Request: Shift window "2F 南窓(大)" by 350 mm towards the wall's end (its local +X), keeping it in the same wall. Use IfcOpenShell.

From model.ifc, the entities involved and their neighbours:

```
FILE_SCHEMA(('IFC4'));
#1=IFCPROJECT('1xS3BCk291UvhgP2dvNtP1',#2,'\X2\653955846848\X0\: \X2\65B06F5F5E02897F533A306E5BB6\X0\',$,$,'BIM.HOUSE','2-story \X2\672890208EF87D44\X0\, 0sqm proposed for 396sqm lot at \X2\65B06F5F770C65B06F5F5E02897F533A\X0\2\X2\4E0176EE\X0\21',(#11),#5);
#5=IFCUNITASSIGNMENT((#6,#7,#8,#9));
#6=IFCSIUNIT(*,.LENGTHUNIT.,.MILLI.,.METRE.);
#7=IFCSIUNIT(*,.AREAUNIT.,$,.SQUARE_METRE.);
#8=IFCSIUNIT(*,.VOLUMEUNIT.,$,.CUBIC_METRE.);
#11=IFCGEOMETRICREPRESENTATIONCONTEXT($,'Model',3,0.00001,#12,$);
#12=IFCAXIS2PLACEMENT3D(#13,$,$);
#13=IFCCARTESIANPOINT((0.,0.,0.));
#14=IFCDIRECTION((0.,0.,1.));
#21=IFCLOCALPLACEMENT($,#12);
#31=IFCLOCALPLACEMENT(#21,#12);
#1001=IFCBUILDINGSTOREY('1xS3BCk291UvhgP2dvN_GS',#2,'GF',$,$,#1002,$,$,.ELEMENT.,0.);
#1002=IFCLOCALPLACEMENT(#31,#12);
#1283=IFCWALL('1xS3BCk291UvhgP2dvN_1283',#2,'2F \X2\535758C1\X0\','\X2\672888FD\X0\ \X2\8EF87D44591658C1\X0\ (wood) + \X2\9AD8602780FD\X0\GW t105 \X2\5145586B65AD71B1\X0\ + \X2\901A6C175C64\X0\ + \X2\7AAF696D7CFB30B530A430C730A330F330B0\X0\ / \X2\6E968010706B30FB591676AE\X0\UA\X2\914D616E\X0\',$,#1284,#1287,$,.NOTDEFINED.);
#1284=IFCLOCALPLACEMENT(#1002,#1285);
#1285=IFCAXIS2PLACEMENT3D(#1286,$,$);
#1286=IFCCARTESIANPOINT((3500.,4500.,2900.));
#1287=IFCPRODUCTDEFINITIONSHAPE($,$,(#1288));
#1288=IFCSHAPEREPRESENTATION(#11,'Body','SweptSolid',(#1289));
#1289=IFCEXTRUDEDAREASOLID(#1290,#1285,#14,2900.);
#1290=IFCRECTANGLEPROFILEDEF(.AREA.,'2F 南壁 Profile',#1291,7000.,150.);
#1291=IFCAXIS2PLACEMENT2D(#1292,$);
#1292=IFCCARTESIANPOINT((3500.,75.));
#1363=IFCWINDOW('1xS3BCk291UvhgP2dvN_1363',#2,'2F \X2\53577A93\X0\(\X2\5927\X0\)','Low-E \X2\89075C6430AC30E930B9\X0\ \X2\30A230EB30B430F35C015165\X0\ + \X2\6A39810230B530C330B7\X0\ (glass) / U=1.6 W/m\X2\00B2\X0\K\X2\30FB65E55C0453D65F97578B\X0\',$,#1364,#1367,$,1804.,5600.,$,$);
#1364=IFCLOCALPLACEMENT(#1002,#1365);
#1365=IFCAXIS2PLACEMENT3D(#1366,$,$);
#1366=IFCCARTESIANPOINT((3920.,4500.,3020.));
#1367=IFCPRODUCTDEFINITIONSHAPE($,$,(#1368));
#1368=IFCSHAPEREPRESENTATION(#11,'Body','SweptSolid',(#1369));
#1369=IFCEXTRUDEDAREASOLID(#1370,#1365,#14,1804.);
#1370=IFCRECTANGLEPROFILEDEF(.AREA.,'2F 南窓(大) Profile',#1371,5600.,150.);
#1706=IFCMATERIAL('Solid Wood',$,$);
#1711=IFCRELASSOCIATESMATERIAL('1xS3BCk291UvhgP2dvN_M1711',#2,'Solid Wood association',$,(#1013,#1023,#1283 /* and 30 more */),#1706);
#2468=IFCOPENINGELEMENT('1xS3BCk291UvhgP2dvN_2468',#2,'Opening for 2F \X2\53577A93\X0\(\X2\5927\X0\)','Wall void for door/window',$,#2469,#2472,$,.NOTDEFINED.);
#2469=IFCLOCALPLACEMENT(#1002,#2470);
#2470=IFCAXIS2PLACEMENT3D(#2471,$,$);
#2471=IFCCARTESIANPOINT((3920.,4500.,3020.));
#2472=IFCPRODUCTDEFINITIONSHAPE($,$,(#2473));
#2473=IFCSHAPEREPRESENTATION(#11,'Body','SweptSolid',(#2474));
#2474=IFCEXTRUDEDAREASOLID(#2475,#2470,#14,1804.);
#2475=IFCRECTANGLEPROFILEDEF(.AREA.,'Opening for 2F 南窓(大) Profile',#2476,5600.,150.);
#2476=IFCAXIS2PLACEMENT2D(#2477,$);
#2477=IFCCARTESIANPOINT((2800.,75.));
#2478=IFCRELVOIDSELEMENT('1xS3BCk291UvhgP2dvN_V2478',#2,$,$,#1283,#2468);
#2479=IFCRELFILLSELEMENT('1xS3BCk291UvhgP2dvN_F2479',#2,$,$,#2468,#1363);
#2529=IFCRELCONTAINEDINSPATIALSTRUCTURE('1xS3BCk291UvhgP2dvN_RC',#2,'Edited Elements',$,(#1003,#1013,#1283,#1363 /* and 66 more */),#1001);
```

```python
import ifcopenshell
import ifcopenshell.api.geometry
import ifcopenshell.util.placement

model = ifcopenshell.open("model.ifc")

window = model.by_guid("1xS3BCk291UvhgP2dvN_1363")
opening = window.FillsVoids[0].RelatingOpeningElement
wall = opening.VoidsElements[0].RelatingBuildingElement

wall_matrix = ifcopenshell.util.placement.get_local_placement(wall.ObjectPlacement)
shift = wall_matrix[:3, 0] * 350.0
before = ifcopenshell.util.placement.get_local_placement(window.ObjectPlacement)[:3, 3].copy()

# The window is not placed relative to its opening, so move both.
for product in (opening, window):
    matrix = ifcopenshell.util.placement.get_local_placement(product.ObjectPlacement)
    matrix[:3, 3] += shift
    ifcopenshell.api.geometry.edit_object_placement(model, product=product, matrix=matrix, is_si=False)

after = ifcopenshell.util.placement.get_local_placement(window.ObjectPlacement)[:3, 3]
print("window moved by", (after - before).round(3) + 0.0)

model.write("model_rev.ifc")
```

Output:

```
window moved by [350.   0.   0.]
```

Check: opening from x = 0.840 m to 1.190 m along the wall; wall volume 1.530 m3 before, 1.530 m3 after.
